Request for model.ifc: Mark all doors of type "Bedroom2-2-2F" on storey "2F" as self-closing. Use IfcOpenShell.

First a look at what the model holds.

```python
import ifcopenshell
import ifcopenshell.util.element

model = ifcopenshell.open("model.ifc")
print(model.schema)
storey = next(s for s in model.by_type("IfcBuildingStorey") if s.Name == "2F")
doors = [e for e in ifcopenshell.util.element.get_decomposition(storey) if e.is_a("IfcDoor")]
seen = {}
for e in doors:
    element_type = ifcopenshell.util.element.get_type(e)
    key = (element_type.Name if element_type != e and element_type else None, ifcopenshell.util.element.get_pset(e, "Pset_DoorCommon", "SelfClosing"))
    seen[key] = seen.get(key, 0) + 1
for (name, value), count in sorted(seen.items(), key=str):
    print(count, "x", name, "|", value)
```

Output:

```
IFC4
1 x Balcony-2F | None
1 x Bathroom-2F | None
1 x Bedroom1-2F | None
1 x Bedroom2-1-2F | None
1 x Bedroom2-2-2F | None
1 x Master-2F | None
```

```python
import ifcopenshell
import ifcopenshell.api.pset
import ifcopenshell.util.element

model = ifcopenshell.open("model.ifc")

storey = next(s for s in model.by_type("IfcBuildingStorey") if s.Name == "2F")
doors = [e for e in ifcopenshell.util.element.get_decomposition(storey) if e.is_a("IfcDoor")]

count = 0
for e in doors:
    element_type = ifcopenshell.util.element.get_type(e)
    if element_type in (None, e) or element_type.Name != "Bedroom2-2-2F":
        continue
    # add_pset returns the element's existing set when there is one.
    pset = ifcopenshell.api.pset.add_pset(model, product=e, name="Pset_DoorCommon")
    ifcopenshell.api.pset.edit_pset(model, pset=pset, properties={"SelfClosing": True})
    count += 1

print(count, "doors updated")

model.write("model_rev.ifc")
```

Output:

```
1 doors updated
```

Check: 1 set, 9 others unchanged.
